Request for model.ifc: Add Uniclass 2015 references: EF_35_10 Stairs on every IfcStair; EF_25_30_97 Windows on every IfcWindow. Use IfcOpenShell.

First a look at what the model holds.

```python
import ifcopenshell

model = ifcopenshell.open("model.ifc")
print(model.schema)
print("classifications:", [c.Name for c in model.by_type("IfcClassification")])
for ifc_class in ("IfcDoor", "IfcRoof", "IfcStair", "IfcWall", "IfcWindow"):
    print(ifc_class, len(model.by_type(ifc_class)))
```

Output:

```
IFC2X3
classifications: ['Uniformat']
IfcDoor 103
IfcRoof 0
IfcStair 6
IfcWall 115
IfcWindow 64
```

```python
import ifcopenshell
import ifcopenshell.api.classification

model = ifcopenshell.open("model.ifc")

# IFC2X3 requires Source and Edition and has no link from the project to the system.
system = model.create_entity("IfcClassification", Source="NBS", Edition="2015", Name="Uniclass 2015")

codes = {
    "IfcStair": ("EF_35_10", "Stairs"),
    "IfcWindow": ("EF_25_30_97", "Windows"),
}
for ifc_class, (code, name) in codes.items():
    products = model.by_type(ifc_class)
    ifcopenshell.api.classification.add_reference(
        model, products=products, classification=system, identification=code, name=name
    )
    print(code, len(products))

model.write("model_rev.ifc")
```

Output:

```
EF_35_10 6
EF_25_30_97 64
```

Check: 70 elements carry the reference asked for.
